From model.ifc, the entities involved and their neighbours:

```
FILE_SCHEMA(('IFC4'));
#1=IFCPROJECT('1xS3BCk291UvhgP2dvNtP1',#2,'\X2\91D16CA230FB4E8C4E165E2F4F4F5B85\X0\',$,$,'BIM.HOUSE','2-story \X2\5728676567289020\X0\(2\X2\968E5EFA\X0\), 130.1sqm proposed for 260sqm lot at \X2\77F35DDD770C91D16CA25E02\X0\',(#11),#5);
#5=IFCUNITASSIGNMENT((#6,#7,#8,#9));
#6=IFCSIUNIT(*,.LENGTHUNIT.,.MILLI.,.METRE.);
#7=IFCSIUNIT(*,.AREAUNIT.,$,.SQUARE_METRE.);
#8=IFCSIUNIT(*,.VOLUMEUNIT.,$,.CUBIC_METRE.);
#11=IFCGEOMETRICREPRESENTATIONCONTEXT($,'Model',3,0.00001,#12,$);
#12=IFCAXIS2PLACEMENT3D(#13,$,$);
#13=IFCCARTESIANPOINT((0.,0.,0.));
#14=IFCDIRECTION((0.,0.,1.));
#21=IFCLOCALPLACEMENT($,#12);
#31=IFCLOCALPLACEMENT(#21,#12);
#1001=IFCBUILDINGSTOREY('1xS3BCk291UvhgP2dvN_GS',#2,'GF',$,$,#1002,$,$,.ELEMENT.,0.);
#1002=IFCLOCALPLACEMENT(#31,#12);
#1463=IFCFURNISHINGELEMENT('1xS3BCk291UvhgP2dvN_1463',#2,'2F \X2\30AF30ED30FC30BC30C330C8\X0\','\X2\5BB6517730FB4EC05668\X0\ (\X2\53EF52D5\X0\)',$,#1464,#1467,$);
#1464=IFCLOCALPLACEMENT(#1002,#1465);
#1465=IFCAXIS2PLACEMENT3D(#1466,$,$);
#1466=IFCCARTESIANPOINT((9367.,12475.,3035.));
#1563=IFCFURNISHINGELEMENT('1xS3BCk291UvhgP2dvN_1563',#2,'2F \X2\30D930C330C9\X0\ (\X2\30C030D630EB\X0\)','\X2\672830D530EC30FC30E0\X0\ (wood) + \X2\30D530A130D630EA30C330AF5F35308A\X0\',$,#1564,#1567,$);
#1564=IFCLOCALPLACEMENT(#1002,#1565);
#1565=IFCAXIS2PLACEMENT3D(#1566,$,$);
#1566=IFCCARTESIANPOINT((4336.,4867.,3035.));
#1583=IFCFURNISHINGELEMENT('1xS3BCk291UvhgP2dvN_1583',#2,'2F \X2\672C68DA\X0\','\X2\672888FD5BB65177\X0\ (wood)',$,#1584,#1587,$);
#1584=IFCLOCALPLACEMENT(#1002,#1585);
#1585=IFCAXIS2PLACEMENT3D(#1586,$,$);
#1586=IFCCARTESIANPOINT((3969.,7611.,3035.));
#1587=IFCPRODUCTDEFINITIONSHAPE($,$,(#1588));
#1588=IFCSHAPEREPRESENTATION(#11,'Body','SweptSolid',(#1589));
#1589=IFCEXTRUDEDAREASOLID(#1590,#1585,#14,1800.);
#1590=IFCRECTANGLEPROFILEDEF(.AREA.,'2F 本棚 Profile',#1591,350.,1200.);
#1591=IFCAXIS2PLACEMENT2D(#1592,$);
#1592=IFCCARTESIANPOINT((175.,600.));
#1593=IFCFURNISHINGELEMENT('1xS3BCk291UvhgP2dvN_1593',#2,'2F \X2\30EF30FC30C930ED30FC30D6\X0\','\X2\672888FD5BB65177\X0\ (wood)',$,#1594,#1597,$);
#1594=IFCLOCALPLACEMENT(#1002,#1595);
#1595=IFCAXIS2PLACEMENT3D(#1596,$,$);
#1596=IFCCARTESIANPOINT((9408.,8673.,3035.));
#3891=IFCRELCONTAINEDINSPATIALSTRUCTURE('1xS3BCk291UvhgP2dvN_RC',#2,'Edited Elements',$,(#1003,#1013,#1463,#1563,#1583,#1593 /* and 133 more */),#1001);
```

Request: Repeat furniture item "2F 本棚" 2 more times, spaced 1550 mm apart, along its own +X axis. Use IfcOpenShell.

```python
import ifcopenshell
import ifcopenshell.api.geometry
import ifcopenshell.api.root
import ifcopenshell.util.element
import ifcopenshell.util.placement
import ifcopenshell.util.unit

model = ifcopenshell.open("model.ifc")
unit_scale = ifcopenshell.util.unit.calculate_unit_scale(model)


def reuse_history(source, copy):
    """copy_class also copies each property set's owner history, people and application; keep the originals."""
    for rel in copy.IsDefinedBy:
        if rel.is_a("IfcRelDefinesByProperties") and (history := rel.RelatingPropertyDefinition.OwnerHistory):
            rel.RelatingPropertyDefinition.OwnerHistory = source.OwnerHistory
            ifcopenshell.util.element.remove_deep2(model, history)


source = model.by_guid("1xS3BCk291UvhgP2dvN_1583")
base = ifcopenshell.util.placement.get_local_placement(source.ObjectPlacement)
step = base[:3, 0] * 1.55 / unit_scale

for i in range(1, 3):
    copy = ifcopenshell.api.root.copy_class(model, product=source)
    copy.Representation = ifcopenshell.util.element.copy_deep(
        model, source.Representation, exclude=["IfcGeometricRepresentationContext", "IfcRepresentationMap"]
    )
    reuse_history(source, copy)
    matrix = base.copy()
    matrix[:3, 3] += i * step
    print("added at", matrix[:3, 3].round(3) + 0.0)
    ifcopenshell.api.geometry.edit_object_placement(model, product=copy, matrix=matrix, is_si=False)

model.write("model_rev.ifc")
```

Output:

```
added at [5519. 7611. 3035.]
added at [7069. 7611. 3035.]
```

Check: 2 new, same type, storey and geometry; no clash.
